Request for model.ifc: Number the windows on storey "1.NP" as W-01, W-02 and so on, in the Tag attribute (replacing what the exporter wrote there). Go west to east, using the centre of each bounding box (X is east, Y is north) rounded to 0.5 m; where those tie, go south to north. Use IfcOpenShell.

First a look at what the model holds.

```python
import ifcopenshell
import ifcopenshell.util.element
import ifcopenshell.util.placement

model = ifcopenshell.open("model.ifc")
print(model.schema)
storey = next(s for s in model.by_type("IfcBuildingStorey") if s.Name == "1.NP")
windows = [e for e in ifcopenshell.util.element.get_decomposition(storey) if e.is_a("IfcWindow")]
for e in sorted(windows, key=lambda e: e.id()):
    origin = ifcopenshell.util.placement.get_local_placement(e.ObjectPlacement)[:3, 3]
    print(e.id(), e.Tag, e.Name, origin.round(2) + 0.0, sep=" | ")
```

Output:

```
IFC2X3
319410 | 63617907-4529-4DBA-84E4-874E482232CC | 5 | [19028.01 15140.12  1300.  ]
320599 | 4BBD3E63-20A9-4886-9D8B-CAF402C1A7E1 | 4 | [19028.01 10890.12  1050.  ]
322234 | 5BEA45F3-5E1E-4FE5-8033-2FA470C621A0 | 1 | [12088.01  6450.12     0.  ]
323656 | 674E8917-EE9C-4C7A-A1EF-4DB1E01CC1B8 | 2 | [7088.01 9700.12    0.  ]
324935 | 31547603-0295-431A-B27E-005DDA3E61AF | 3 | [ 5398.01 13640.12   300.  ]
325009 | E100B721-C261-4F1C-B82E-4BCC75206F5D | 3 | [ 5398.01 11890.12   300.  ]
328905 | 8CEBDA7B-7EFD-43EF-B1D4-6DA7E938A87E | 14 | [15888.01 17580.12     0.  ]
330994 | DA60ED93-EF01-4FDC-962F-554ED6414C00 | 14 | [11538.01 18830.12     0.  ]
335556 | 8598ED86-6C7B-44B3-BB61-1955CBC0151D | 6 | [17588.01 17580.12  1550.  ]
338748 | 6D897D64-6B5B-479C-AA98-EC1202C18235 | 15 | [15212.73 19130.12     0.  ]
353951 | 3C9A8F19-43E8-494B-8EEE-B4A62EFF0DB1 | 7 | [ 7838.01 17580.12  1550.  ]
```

```python
import ifcopenshell
import ifcopenshell.geom
import ifcopenshell.util.element
import ifcopenshell.util.shape

model = ifcopenshell.open("model.ifc")
settings = ifcopenshell.geom.settings()
settings.set("use-world-coords", True)


def centre(element):
    shape = ifcopenshell.geom.create_shape(settings, element)
    return ifcopenshell.util.shape.get_bbox_centroid(shape.geometry)


storey = next(s for s in model.by_type("IfcBuildingStorey") if s.Name == "1.NP")
windows = [e for e in ifcopenshell.util.element.get_decomposition(storey) if e.is_a("IfcWindow")]

# Insertion points can sit at a corner or the storey origin, so sort by the geometry (in metres).
centres = {e: centre(e) for e in windows}
windows.sort(key=lambda e: (round(centres[e][0] / 0.5), centres[e][1]))

for i, e in enumerate(windows, start=1):
    number = f"W-{i:02d}"
    e.Tag = number
    print(e.id(), number)

model.write("model_v2.ifc")
```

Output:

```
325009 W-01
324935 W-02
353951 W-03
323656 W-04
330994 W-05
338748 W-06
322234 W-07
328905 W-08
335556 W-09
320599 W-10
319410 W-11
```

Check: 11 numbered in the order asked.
